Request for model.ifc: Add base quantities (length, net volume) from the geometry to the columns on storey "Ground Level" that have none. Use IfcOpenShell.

First a look at what the model holds.

```python
import ifcopenshell
import ifcopenshell.util.element
import ifcopenshell.util.unit

model = ifcopenshell.open("model.ifc")
print(model.schema)
for unit_type in ("LENGTHUNIT", "AREAUNIT", "VOLUMEUNIT"):
    print(unit_type, ifcopenshell.util.unit.calculate_unit_scale(model, unit_type))
storey = next(s for s in model.by_type("IfcBuildingStorey") if s.Name == "Ground Level")
columns = [e for e in ifcopenshell.util.element.get_decomposition(storey) if e.is_a("IfcColumn")]
for e in sorted(columns, key=lambda e: e.id()):
    print(e.id(), e.is_a(), e.Name, list(ifcopenshell.util.element.get_psets(e, qtos_only=True)), sep=" | ")
```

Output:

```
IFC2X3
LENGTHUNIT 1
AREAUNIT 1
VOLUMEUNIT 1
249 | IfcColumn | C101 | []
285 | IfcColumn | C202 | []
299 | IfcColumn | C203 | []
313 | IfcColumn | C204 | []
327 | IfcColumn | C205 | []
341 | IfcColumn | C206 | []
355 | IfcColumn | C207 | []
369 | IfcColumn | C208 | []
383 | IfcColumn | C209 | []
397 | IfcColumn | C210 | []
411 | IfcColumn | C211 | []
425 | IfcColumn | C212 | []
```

```python
import ifcopenshell
import ifcopenshell.api.pset
import ifcopenshell.geom
import ifcopenshell.util.element
import ifcopenshell.util.shape
import ifcopenshell.util.unit

model = ifcopenshell.open("model.ifc")
unit_scale = ifcopenshell.util.unit.calculate_unit_scale(model)
volume_scale = ifcopenshell.util.unit.calculate_unit_scale(model, "VOLUMEUNIT")
settings = ifcopenshell.geom.settings()

storey = next(s for s in model.by_type("IfcBuildingStorey") if s.Name == "Ground Level")
columns = [e for e in ifcopenshell.util.element.get_decomposition(storey) if e.is_a("IfcColumn")]

for e in sorted(columns, key=lambda e: e.id()):
    if ifcopenshell.util.element.get_psets(e, qtos_only=True, should_inherit=False):
        continue
    # Geometry comes back in metres, in the element's own axes.
    shape = ifcopenshell.geom.create_shape(settings, e)
    values = {
        "Length": ifcopenshell.util.shape.get_z(shape.geometry) / unit_scale,
        "NetVolume": ifcopenshell.util.shape.get_volume(shape.geometry) / volume_scale,
    }
    qto = ifcopenshell.api.pset.add_qto(model, product=e, name="BaseQuantities")
    ifcopenshell.api.pset.edit_qto(model, qto=qto, properties=values)
    print(e.id(), {k: round(v, 3) for k, v in values.items()})

model.write("model_updated.ifc")
```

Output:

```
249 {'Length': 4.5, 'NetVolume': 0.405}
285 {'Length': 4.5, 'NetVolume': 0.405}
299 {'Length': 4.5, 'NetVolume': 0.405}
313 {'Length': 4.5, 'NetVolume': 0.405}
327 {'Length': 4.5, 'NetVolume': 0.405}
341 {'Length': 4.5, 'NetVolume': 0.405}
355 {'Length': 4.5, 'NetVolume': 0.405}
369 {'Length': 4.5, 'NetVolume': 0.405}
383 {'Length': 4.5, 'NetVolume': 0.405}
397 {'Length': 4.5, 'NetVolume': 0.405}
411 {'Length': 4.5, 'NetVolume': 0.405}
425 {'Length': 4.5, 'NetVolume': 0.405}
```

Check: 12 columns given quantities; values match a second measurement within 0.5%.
